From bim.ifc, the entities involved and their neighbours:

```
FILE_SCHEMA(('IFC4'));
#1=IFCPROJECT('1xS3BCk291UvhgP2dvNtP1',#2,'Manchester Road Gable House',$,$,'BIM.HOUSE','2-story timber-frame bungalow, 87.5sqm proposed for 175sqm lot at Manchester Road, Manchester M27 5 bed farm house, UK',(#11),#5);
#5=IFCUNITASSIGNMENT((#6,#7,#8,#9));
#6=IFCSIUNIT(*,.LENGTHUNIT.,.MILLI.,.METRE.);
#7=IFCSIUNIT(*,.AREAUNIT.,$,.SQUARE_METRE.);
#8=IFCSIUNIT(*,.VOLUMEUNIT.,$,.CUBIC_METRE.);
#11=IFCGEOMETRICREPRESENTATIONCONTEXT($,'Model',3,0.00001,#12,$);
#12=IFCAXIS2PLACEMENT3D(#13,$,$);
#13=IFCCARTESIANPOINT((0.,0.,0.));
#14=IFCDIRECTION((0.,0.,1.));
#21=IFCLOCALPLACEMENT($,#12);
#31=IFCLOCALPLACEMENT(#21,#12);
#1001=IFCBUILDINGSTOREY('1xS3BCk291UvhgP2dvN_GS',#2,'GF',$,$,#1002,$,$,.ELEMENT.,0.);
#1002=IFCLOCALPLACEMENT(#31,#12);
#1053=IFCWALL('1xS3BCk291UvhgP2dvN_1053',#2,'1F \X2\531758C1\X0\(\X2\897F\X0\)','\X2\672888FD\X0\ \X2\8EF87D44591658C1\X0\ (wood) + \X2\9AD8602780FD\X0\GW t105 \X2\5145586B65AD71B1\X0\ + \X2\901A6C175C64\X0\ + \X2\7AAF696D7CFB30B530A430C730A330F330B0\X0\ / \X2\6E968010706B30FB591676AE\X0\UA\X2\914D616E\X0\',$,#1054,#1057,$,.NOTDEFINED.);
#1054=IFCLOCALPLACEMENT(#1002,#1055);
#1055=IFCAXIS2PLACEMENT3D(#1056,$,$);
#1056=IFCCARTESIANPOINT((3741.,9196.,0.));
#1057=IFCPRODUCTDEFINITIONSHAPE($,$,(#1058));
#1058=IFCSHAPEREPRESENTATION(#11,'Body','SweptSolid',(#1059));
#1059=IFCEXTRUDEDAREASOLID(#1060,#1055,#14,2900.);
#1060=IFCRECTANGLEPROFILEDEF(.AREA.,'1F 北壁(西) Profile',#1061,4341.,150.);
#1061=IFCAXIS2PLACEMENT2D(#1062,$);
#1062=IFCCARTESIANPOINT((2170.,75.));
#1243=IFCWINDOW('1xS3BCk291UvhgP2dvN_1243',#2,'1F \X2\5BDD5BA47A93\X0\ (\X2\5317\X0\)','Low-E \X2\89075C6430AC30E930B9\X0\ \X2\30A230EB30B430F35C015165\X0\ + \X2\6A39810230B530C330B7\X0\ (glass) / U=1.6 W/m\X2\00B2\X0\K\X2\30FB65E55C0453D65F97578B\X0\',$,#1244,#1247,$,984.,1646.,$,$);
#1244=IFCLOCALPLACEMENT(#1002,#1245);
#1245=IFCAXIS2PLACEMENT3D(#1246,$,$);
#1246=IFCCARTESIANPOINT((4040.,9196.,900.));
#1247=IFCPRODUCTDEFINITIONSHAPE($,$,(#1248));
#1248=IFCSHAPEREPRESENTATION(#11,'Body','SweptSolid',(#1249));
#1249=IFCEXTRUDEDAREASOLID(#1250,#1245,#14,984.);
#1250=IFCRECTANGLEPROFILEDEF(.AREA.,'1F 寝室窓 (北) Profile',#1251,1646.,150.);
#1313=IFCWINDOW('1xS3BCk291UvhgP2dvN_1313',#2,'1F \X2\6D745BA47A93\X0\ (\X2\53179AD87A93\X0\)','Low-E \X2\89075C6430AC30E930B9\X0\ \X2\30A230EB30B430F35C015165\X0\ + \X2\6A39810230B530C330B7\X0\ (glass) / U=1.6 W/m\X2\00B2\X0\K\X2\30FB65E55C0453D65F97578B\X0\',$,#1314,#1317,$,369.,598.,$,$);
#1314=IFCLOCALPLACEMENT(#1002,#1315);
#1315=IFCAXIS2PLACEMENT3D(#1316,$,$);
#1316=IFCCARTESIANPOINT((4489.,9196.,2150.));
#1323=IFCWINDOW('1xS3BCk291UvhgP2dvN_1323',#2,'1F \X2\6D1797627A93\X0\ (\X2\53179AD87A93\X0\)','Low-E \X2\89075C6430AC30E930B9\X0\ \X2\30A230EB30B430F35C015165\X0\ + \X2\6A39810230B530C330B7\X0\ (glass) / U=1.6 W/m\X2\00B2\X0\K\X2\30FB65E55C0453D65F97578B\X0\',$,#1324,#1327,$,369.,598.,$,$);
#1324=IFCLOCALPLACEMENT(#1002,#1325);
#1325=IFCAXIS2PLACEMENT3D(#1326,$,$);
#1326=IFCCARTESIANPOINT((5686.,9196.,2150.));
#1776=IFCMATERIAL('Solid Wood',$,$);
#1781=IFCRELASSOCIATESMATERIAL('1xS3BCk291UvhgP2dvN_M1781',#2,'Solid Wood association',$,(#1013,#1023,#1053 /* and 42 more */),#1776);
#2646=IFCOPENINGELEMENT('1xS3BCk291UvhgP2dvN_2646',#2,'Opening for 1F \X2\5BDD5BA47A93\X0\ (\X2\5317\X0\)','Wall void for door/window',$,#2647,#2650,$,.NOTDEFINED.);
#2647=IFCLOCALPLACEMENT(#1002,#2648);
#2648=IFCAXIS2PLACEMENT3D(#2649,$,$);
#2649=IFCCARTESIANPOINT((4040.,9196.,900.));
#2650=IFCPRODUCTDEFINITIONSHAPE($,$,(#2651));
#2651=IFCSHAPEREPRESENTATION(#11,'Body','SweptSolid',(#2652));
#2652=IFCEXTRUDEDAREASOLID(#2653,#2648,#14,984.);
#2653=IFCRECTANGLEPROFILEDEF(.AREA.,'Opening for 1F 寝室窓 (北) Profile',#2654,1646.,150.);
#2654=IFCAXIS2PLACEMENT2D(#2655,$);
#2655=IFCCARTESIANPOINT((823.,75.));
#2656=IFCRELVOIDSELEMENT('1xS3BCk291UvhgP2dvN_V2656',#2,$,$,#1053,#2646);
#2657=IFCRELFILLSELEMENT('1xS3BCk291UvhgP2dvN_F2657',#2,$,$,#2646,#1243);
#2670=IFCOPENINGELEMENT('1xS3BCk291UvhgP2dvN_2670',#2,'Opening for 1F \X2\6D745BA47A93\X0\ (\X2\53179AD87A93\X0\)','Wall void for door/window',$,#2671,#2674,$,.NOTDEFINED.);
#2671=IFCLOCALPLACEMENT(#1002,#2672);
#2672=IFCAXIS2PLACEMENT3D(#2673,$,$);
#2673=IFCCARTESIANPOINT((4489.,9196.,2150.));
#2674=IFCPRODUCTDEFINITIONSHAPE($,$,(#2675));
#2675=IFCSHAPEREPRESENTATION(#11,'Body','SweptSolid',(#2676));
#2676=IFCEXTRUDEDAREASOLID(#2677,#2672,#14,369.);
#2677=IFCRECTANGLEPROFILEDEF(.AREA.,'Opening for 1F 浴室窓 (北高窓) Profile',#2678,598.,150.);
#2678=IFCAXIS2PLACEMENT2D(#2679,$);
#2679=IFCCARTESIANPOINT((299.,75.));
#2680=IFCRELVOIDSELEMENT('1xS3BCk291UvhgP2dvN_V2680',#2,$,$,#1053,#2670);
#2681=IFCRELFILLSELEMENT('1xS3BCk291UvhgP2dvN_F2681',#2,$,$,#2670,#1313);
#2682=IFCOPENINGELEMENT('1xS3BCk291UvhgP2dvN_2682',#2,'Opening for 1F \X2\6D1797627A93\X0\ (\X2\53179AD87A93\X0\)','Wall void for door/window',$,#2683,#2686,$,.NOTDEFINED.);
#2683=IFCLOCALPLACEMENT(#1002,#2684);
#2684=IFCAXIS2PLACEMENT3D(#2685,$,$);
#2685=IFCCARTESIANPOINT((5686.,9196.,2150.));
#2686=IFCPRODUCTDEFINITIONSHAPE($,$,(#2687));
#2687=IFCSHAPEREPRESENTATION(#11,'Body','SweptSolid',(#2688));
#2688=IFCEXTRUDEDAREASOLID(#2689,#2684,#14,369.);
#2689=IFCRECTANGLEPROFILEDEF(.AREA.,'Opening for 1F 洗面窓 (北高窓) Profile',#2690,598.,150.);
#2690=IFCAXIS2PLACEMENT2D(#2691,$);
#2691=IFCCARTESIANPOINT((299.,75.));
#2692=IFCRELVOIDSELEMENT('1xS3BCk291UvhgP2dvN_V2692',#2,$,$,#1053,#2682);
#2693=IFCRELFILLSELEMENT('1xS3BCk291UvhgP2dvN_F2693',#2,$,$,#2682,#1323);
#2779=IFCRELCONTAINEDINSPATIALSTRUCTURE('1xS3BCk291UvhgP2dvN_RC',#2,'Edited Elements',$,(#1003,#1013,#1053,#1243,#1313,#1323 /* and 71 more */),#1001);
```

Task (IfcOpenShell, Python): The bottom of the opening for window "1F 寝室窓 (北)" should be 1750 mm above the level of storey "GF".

```python
import numpy as np
import ifcopenshell
import ifcopenshell.api.geometry
import ifcopenshell.geom
import ifcopenshell.util.element
import ifcopenshell.util.placement
import ifcopenshell.util.shape
import ifcopenshell.util.unit

model = ifcopenshell.open("bim.ifc")
unit_scale = ifcopenshell.util.unit.calculate_unit_scale(model)

window = model.by_guid("1xS3BCk291UvhgP2dvN_1243")
opening = window.FillsVoids[0].RelatingOpeningElement
storey = ifcopenshell.util.element.get_container(window, ifc_class="IfcBuildingStorey")
level = ifcopenshell.util.placement.get_local_placement(storey.ObjectPlacement)[2, 3]

# The opening's origin need not be at the sill, so measure its lowest point.
shape = ifcopenshell.geom.create_shape(ifcopenshell.geom.settings(), opening)
bottom = ifcopenshell.util.shape.get_shape_bottom_elevation(shape, shape.geometry) / unit_scale
dz = level + 1750.0 - bottom

shift = np.array([0.0, 0.0, dz])
# The window is not placed relative to its opening, so move both.
for product in (opening, window):
    matrix = ifcopenshell.util.placement.get_local_placement(product.ObjectPlacement)
    matrix[:3, 3] += shift
    ifcopenshell.api.geometry.edit_object_placement(model, product=product, matrix=matrix, is_si=False)

print(f"moved by {dz * unit_scale:+.3f} m")

model.write("bim_v2.ifc")
```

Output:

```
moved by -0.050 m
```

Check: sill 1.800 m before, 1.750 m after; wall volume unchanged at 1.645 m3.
